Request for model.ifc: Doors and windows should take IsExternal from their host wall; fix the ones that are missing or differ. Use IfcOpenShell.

First a look at what the model holds.

```python
import ifcopenshell
import ifcopenshell.util.element

model = ifcopenshell.open("model.ifc")
print(model.schema)
seen = {}
for e in model.by_type("IfcDoor") + model.by_type("IfcWindow"):
    if not e.FillsVoids:
        continue
    host = e.FillsVoids[0].RelatingOpeningElement.VoidsElements[0].RelatingBuildingElement
    own = ifcopenshell.util.element.get_pset(e, f"Pset_{e.is_a()[3:].removesuffix('StandardCase')}Common", "IsExternal")
    wall = ifcopenshell.util.element.get_pset(host, "Pset_WallCommon", "IsExternal")
    seen[e.is_a(), own, wall] = seen.get((e.is_a(), own, wall), 0) + 1
for (cls, own, wall), count in sorted(seen.items(), key=str):
    print(count, cls, "IsExternal:", own, "| host wall:", wall)
```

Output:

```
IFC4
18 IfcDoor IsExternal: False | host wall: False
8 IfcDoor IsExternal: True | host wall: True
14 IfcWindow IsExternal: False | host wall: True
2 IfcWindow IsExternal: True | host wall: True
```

```python
import ifcopenshell
import ifcopenshell.api.pset
import ifcopenshell.util.element

model = ifcopenshell.open("model.ifc")

count = 0
for ifc_class, pset_name in (("IfcDoor", "Pset_DoorCommon"), ("IfcWindow", "Pset_WindowCommon")):
    for e in model.by_type(ifc_class):
        if not e.FillsVoids:
            continue
        host = e.FillsVoids[0].RelatingOpeningElement.VoidsElements[0].RelatingBuildingElement
        external = ifcopenshell.util.element.get_pset(host, "Pset_WallCommon", "IsExternal")
        if external is None or ifcopenshell.util.element.get_pset(e, pset_name, "IsExternal") == external:
            continue
        pset = ifcopenshell.api.pset.add_pset(model, product=e, name=pset_name)
        ifcopenshell.api.pset.edit_pset(model, pset=pset, properties={"IsExternal": external})
        count += 1

print(count, "updated")

model.write("model_rev.ifc")
```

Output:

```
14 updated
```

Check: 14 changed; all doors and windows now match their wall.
